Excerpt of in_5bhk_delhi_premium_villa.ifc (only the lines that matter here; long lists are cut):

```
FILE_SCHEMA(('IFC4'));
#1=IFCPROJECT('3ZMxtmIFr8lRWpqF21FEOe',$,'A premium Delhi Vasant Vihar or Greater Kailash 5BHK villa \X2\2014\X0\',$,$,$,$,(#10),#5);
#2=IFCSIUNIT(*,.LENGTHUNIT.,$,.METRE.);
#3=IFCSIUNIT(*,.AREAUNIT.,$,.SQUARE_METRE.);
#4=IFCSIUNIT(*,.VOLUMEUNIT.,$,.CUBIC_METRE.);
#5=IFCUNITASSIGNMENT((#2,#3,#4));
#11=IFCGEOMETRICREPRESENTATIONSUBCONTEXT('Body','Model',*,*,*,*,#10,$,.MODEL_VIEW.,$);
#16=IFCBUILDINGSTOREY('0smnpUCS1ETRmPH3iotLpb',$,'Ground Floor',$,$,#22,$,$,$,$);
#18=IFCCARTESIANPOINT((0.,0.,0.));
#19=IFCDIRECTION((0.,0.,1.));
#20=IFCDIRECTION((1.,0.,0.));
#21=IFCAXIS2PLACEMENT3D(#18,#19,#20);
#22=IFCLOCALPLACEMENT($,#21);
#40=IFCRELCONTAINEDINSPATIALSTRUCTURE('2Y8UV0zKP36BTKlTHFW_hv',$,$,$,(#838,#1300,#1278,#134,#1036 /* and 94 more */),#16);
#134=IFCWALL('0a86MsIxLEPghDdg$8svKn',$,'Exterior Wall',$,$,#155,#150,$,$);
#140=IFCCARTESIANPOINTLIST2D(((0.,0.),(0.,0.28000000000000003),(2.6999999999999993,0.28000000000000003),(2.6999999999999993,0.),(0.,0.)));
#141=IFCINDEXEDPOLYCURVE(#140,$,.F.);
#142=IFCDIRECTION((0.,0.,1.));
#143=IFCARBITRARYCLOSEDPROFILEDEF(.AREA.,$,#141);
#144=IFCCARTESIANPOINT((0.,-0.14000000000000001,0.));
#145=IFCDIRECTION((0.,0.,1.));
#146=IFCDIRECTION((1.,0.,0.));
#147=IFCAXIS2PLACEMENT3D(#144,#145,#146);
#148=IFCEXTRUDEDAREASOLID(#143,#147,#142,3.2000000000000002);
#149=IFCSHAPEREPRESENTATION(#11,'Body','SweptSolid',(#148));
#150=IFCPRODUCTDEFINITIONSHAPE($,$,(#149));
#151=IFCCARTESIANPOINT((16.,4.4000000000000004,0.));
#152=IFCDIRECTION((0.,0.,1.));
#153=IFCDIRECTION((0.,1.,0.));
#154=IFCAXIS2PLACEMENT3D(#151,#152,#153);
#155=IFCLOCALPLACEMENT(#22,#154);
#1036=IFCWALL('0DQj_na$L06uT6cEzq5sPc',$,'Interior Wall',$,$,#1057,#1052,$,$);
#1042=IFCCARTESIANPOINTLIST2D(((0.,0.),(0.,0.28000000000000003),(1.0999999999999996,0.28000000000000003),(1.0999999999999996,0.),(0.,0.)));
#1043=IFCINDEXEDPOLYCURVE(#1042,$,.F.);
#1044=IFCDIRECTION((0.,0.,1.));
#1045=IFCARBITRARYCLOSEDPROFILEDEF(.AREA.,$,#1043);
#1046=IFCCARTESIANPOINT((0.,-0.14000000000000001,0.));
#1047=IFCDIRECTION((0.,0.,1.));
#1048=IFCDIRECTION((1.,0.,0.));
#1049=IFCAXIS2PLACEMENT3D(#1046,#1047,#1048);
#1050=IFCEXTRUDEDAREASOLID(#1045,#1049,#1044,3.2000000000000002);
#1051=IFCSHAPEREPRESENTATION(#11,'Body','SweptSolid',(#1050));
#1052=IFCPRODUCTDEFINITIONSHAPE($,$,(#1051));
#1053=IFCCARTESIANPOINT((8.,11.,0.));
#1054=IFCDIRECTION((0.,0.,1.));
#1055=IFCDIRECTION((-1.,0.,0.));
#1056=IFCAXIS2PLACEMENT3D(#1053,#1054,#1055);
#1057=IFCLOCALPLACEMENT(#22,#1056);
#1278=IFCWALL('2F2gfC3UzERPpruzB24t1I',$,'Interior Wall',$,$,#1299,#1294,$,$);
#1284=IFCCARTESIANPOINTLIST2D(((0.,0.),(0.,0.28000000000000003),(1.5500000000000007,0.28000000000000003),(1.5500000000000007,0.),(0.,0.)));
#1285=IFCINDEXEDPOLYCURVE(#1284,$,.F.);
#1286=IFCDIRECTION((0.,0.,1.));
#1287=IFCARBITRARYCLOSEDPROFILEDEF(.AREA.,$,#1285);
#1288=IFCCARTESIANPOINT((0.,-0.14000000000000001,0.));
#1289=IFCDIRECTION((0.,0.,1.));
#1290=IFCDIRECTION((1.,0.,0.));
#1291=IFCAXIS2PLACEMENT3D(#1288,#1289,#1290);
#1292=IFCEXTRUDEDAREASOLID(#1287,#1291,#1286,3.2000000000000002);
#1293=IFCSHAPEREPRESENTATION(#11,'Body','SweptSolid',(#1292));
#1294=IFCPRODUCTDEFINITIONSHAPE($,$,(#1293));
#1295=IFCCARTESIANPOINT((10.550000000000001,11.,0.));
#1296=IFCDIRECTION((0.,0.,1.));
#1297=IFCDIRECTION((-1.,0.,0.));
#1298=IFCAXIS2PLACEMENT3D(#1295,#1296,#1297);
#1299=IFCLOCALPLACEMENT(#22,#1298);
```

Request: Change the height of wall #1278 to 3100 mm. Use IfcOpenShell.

```python
import ifcopenshell
import ifcopenshell.geom
import ifcopenshell.util.representation
import ifcopenshell.util.shape
import ifcopenshell.util.unit

model = ifcopenshell.open("in_5bhk_delhi_premium_villa.ifc")
unit_scale = ifcopenshell.util.unit.calculate_unit_scale(model)
settings = ifcopenshell.geom.settings()


def volume(element):
    """Net volume in cubic metres, openings subtracted."""
    shape = ifcopenshell.geom.create_shape(settings, element)
    return ifcopenshell.util.shape.get_volume(shape.geometry)


wall = model.by_id(1278)
before = volume(wall)

body = ifcopenshell.util.representation.get_representation(wall, "Model", "Body")
solid = body.Items[0]
old_height = solid.Depth
solid.Depth = 3.1 / unit_scale
after = volume(wall)

print(f"height {old_height:g} -> {solid.Depth:g}, volume {before:.3f} -> {after:.3f} m3")

model.write("in_5bhk_delhi_premium_villa_edited.ifc")
```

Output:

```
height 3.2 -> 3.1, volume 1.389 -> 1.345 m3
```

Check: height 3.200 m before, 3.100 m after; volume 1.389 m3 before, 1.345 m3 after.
